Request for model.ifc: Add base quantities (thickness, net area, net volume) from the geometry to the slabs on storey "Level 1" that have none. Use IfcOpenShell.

First a look at what the model holds.

```python
import ifcopenshell
import ifcopenshell.util.element
import ifcopenshell.util.unit

model = ifcopenshell.open("model.ifc")
print(model.schema)
for unit_type in ("LENGTHUNIT", "AREAUNIT", "VOLUMEUNIT"):
    print(unit_type, ifcopenshell.util.unit.calculate_unit_scale(model, unit_type))
storey = next(s for s in model.by_type("IfcBuildingStorey") if s.Name == "Level 1")
slabs = [e for e in ifcopenshell.util.element.get_decomposition(storey) if e.is_a("IfcSlab")]
for e in sorted(slabs, key=lambda e: e.id()):
    print(e.id(), e.is_a(), e.Name, list(ifcopenshell.util.element.get_psets(e, qtos_only=True)), sep=" | ")
```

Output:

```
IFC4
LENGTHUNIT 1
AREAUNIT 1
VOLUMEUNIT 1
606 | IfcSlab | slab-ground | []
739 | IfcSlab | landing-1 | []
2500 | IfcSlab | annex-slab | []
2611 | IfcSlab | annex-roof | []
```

```python
import ifcopenshell
import ifcopenshell.api.pset
import ifcopenshell.geom
import ifcopenshell.util.element
import ifcopenshell.util.shape
import ifcopenshell.util.unit

model = ifcopenshell.open("model.ifc")
unit_scale = ifcopenshell.util.unit.calculate_unit_scale(model)
area_scale = ifcopenshell.util.unit.calculate_unit_scale(model, "AREAUNIT")
volume_scale = ifcopenshell.util.unit.calculate_unit_scale(model, "VOLUMEUNIT")
settings = ifcopenshell.geom.settings()

storey = next(s for s in model.by_type("IfcBuildingStorey") if s.Name == "Level 1")
slabs = [e for e in ifcopenshell.util.element.get_decomposition(storey) if e.is_a("IfcSlab")]

for e in sorted(slabs, key=lambda e: e.id()):
    if ifcopenshell.util.element.get_psets(e, qtos_only=True, should_inherit=False):
        continue
    # Geometry comes back in metres, in the element's own axes.
    shape = ifcopenshell.geom.create_shape(settings, e)
    values = {
        "Width": ifcopenshell.util.shape.get_z(shape.geometry) / unit_scale,
        "NetArea": ifcopenshell.util.shape.get_footprint_area(shape.geometry) / area_scale,
        "NetVolume": ifcopenshell.util.shape.get_volume(shape.geometry) / volume_scale,
    }
    qto = ifcopenshell.api.pset.add_qto(model, product=e, name="Qto_SlabBaseQuantities")
    ifcopenshell.api.pset.edit_qto(model, qto=qto, properties=values)
    print(e.id(), {k: round(v, 3) for k, v in values.items()})

model.write("model_rev.ifc")
```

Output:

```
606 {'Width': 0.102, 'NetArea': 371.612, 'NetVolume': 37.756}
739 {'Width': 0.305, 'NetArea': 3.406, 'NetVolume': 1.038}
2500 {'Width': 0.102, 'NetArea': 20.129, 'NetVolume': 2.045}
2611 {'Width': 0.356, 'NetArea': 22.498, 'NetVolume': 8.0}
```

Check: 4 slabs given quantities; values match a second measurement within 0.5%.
